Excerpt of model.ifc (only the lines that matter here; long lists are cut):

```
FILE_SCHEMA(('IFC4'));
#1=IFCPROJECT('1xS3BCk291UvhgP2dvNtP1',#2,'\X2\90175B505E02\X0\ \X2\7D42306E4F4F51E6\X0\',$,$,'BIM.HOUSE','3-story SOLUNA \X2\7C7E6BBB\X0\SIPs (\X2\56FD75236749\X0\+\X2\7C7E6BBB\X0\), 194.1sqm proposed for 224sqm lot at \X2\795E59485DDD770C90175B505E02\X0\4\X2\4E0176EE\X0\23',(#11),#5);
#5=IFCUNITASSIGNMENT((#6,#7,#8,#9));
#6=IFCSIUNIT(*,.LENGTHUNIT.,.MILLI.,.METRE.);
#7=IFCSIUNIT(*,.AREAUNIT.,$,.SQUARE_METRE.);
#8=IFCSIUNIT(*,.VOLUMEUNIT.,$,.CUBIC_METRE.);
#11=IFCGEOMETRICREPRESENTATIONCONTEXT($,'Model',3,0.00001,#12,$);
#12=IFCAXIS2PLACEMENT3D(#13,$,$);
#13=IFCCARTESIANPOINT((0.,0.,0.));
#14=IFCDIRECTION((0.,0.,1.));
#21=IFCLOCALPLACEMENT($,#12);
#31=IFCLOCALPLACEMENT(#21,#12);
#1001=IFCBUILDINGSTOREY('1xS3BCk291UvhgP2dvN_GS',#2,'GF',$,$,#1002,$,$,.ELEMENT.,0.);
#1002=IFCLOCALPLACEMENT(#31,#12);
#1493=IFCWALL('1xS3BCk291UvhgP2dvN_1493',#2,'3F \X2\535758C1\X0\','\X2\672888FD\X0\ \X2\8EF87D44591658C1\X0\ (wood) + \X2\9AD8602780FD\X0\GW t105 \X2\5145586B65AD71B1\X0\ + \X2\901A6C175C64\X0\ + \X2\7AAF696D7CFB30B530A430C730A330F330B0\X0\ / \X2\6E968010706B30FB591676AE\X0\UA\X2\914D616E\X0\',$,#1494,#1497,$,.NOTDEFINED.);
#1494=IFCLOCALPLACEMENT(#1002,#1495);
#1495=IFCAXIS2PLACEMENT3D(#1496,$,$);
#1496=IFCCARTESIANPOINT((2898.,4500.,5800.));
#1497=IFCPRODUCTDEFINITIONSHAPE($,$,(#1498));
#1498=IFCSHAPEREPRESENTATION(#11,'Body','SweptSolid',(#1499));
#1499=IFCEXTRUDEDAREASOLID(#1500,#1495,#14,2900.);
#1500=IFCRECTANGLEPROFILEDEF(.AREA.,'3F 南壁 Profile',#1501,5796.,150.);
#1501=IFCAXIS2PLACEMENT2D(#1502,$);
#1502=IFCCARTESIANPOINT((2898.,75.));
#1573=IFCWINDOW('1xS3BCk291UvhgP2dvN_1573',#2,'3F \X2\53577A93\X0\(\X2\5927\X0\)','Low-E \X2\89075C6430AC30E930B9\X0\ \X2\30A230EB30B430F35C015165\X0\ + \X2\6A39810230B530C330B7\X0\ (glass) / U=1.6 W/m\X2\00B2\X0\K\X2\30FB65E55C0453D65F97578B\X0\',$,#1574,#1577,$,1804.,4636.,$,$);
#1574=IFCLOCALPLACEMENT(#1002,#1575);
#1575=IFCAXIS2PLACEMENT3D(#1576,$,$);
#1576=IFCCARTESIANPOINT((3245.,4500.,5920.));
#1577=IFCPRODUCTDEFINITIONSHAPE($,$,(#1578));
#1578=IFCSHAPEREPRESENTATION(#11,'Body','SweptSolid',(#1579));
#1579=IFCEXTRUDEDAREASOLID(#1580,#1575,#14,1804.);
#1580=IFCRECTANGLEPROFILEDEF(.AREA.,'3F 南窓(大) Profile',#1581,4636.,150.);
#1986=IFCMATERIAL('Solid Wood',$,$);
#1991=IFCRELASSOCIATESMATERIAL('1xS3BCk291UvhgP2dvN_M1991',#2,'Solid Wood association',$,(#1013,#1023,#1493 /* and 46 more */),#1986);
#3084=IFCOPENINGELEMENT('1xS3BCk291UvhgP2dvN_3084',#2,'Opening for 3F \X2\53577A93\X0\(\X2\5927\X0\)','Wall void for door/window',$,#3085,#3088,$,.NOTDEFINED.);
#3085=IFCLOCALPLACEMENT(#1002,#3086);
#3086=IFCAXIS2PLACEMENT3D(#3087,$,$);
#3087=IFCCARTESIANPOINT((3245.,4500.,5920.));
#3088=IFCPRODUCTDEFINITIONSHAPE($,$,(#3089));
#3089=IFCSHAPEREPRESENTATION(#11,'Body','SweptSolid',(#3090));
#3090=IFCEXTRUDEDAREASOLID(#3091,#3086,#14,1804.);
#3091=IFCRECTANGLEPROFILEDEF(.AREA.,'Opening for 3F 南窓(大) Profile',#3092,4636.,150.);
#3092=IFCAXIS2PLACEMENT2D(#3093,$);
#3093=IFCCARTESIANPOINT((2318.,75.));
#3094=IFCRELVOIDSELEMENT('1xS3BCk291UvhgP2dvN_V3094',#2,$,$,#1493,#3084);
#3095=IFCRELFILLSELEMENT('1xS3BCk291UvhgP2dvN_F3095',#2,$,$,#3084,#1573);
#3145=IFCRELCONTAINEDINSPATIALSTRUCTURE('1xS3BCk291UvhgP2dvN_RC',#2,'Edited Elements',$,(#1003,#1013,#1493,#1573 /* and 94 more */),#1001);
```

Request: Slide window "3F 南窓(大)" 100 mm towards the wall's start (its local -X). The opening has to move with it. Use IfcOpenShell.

```python
import ifcopenshell
import ifcopenshell.api.geometry
import ifcopenshell.util.placement

model = ifcopenshell.open("model.ifc")

window = model.by_guid("1xS3BCk291UvhgP2dvN_1573")
opening = window.FillsVoids[0].RelatingOpeningElement
wall = opening.VoidsElements[0].RelatingBuildingElement

wall_matrix = ifcopenshell.util.placement.get_local_placement(wall.ObjectPlacement)
shift = wall_matrix[:3, 0] * -100.0
before = ifcopenshell.util.placement.get_local_placement(window.ObjectPlacement)[:3, 3].copy()

# The window is not placed relative to its opening, so move both.
for product in (opening, window):
    matrix = ifcopenshell.util.placement.get_local_placement(product.ObjectPlacement)
    matrix[:3, 3] += shift
    ifcopenshell.api.geometry.edit_object_placement(model, product=product, matrix=matrix, is_si=False)

after = ifcopenshell.util.placement.get_local_placement(window.ObjectPlacement)[:3, 3]
print("window moved by", (after - before).round(3) + 0.0)

model.write("model-out.ifc")
```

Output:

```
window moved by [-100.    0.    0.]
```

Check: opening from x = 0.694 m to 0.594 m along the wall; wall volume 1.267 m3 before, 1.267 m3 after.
